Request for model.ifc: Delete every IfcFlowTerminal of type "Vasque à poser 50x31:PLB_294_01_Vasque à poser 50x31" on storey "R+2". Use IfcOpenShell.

First a look at what the model holds.

```python
import ifcopenshell
import ifcopenshell.util.element

model = ifcopenshell.open("model.ifc")
print(model.schema)
storey = next(s for s in model.by_type("IfcBuildingStorey") if s.Name == "R+2")
terminals = [e for e in ifcopenshell.util.element.get_decomposition(storey) if e.is_a("IfcFlowTerminal")]
seen = {}
for e in terminals:
    element_type = ifcopenshell.util.element.get_type(e)
    name = element_type.Name if element_type not in (None, e) else None
    seen[name] = seen.get(name, 0) + 1
for name, count in sorted(seen.items(), key=str):
    print(count, "x", name)
```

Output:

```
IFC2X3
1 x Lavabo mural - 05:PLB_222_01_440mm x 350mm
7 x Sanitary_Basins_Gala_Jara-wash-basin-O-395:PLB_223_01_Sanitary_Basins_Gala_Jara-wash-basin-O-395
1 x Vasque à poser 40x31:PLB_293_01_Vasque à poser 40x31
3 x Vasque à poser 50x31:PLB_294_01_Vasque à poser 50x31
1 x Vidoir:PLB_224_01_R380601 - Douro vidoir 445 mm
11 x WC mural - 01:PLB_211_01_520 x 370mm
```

```python
import ifcopenshell
import ifcopenshell.api.root
import ifcopenshell.util.element

model = ifcopenshell.open("model.ifc")

storey = next(s for s in model.by_type("IfcBuildingStorey") if s.Name == "R+2")
terminals = [e for e in ifcopenshell.util.element.get_decomposition(storey) if e.is_a("IfcFlowTerminal")]
targets = [e for e in terminals if (t := ifcopenshell.util.element.get_type(e)) not in (None, e) and t.Name == "Vasque à poser 50x31:PLB_294_01_Vasque à poser 50x31"]

for e in targets:
    ifcopenshell.api.root.remove_product(model, product=e)
print(len(targets), "removed")

model.write("model_edited.ifc")
```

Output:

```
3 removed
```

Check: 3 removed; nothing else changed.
